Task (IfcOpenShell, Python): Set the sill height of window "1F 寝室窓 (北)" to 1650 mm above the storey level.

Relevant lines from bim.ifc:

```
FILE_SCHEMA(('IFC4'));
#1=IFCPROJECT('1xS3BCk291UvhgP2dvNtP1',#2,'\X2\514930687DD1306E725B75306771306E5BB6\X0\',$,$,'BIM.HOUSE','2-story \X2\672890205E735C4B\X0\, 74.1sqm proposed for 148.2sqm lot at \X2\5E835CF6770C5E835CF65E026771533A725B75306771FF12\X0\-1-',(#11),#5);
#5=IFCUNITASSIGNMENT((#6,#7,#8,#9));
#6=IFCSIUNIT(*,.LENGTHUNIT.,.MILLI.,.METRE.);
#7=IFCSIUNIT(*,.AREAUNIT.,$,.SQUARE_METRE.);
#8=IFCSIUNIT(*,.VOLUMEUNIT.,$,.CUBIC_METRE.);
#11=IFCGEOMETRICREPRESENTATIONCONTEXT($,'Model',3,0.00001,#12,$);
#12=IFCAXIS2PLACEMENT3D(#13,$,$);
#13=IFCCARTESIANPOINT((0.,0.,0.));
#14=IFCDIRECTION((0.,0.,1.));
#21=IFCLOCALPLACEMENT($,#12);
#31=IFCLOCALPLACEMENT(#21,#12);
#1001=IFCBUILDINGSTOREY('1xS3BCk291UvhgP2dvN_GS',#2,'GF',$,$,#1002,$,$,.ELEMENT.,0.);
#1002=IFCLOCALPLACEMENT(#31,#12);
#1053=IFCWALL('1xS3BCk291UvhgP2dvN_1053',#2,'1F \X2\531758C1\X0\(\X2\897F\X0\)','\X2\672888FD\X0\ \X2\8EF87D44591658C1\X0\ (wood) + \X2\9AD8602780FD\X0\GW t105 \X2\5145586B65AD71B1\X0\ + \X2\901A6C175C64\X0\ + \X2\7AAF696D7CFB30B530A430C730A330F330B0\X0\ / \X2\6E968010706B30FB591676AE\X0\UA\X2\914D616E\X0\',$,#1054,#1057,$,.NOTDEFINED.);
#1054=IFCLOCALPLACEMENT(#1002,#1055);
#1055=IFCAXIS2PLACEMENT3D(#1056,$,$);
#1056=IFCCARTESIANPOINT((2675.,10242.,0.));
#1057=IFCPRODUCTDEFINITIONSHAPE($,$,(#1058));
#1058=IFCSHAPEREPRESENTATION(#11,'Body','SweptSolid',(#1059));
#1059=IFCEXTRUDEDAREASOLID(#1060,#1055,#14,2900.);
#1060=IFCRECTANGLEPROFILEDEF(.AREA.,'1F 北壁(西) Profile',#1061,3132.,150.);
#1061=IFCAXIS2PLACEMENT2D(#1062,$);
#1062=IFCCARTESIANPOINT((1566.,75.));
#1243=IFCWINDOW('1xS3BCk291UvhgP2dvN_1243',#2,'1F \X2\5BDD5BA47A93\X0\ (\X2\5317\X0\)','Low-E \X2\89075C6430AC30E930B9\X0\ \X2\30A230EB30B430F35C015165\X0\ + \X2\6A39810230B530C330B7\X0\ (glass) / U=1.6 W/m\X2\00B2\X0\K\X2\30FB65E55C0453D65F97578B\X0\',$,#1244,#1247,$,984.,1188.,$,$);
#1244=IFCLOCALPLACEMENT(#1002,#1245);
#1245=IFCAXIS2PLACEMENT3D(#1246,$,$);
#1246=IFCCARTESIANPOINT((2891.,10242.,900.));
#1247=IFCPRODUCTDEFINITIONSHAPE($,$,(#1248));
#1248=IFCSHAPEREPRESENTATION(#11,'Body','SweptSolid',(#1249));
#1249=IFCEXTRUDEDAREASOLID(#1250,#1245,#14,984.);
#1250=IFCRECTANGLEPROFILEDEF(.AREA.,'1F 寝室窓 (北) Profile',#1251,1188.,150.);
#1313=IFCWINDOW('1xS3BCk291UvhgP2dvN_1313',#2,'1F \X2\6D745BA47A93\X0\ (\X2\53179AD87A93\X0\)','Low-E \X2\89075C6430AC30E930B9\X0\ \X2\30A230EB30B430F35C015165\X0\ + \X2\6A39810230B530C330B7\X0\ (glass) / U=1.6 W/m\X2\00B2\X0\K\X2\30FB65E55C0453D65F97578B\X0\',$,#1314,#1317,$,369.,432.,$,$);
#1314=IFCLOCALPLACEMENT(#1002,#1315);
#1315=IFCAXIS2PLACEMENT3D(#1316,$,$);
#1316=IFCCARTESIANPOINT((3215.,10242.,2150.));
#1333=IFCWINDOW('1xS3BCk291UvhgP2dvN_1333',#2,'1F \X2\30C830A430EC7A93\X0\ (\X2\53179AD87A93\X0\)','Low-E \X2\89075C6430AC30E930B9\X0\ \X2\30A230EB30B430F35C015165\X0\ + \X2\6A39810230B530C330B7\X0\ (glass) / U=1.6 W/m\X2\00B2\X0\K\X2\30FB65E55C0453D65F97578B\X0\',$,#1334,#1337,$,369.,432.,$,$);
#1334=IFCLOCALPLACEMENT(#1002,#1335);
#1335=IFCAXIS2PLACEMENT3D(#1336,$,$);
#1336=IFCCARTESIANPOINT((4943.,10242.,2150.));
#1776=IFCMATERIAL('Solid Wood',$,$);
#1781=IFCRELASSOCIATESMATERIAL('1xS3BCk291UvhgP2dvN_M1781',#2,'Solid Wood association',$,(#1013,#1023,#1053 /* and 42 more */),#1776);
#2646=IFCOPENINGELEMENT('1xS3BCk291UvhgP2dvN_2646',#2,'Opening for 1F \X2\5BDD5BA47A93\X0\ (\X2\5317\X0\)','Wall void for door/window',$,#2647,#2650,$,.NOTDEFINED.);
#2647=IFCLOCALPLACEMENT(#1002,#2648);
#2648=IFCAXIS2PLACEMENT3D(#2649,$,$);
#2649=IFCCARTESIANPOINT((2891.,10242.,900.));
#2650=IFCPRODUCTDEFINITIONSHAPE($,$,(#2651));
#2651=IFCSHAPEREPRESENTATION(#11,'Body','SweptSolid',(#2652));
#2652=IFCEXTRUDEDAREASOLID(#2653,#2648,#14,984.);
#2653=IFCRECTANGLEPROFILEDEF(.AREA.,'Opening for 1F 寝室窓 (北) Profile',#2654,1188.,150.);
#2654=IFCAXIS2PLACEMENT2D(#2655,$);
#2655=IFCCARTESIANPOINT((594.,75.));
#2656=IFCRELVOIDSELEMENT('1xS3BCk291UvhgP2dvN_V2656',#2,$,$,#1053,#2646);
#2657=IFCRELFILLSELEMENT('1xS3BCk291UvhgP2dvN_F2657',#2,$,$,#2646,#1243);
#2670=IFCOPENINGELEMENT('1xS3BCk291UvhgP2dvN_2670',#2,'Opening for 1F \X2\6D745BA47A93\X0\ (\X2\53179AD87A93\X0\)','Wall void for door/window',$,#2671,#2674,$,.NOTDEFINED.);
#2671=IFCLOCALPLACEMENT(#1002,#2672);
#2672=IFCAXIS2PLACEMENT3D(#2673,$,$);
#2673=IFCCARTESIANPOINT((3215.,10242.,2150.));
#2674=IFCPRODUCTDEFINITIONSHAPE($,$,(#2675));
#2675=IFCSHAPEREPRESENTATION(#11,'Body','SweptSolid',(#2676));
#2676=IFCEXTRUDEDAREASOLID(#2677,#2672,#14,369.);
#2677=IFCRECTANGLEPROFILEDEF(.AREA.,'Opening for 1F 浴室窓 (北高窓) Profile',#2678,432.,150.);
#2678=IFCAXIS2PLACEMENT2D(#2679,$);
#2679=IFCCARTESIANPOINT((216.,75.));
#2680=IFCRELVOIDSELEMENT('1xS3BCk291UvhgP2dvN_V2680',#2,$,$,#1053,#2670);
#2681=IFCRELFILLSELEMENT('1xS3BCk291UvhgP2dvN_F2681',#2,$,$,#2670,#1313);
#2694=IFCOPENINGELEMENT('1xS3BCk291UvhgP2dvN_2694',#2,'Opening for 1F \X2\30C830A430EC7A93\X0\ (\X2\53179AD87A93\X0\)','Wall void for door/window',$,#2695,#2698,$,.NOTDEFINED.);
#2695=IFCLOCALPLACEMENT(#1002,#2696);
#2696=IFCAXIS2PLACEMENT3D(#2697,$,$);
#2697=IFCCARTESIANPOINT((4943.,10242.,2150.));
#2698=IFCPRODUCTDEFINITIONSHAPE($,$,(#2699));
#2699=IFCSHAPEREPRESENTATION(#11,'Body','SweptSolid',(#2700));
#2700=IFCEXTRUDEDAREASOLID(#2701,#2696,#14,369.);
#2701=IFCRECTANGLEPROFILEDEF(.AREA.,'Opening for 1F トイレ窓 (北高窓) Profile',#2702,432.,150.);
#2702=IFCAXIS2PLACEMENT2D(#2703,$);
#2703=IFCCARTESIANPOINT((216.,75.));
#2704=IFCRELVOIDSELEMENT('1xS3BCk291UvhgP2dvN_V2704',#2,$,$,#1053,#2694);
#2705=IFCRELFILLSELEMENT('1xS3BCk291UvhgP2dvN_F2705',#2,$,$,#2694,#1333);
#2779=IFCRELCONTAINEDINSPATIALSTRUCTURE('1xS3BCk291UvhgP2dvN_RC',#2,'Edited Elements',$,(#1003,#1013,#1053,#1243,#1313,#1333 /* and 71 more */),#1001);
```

```python
import numpy as np
import ifcopenshell
import ifcopenshell.api.geometry
import ifcopenshell.geom
import ifcopenshell.util.element
import ifcopenshell.util.placement
import ifcopenshell.util.shape
import ifcopenshell.util.unit

model = ifcopenshell.open("bim.ifc")
unit_scale = ifcopenshell.util.unit.calculate_unit_scale(model)

window = model.by_guid("1xS3BCk291UvhgP2dvN_1243")
opening = window.FillsVoids[0].RelatingOpeningElement
storey = ifcopenshell.util.element.get_container(window, ifc_class="IfcBuildingStorey")
level = ifcopenshell.util.placement.get_local_placement(storey.ObjectPlacement)[2, 3]

# The opening's origin need not be at the sill, so measure its lowest point.
shape = ifcopenshell.geom.create_shape(ifcopenshell.geom.settings(), opening)
bottom = ifcopenshell.util.shape.get_shape_bottom_elevation(shape, shape.geometry) / unit_scale
dz = level + 1650.0 - bottom

shift = np.array([0.0, 0.0, dz])
# The window is not placed relative to its opening, so move both.
for product in (opening, window):
    matrix = ifcopenshell.util.placement.get_local_placement(product.ObjectPlacement)
    matrix[:3, 3] += shift
    ifcopenshell.api.geometry.edit_object_placement(model, product=product, matrix=matrix, is_si=False)

print(f"moved by {dz * unit_scale:+.3f} m")

model.write("bim-out.ifc")
```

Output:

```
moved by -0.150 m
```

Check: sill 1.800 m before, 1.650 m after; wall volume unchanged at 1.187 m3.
